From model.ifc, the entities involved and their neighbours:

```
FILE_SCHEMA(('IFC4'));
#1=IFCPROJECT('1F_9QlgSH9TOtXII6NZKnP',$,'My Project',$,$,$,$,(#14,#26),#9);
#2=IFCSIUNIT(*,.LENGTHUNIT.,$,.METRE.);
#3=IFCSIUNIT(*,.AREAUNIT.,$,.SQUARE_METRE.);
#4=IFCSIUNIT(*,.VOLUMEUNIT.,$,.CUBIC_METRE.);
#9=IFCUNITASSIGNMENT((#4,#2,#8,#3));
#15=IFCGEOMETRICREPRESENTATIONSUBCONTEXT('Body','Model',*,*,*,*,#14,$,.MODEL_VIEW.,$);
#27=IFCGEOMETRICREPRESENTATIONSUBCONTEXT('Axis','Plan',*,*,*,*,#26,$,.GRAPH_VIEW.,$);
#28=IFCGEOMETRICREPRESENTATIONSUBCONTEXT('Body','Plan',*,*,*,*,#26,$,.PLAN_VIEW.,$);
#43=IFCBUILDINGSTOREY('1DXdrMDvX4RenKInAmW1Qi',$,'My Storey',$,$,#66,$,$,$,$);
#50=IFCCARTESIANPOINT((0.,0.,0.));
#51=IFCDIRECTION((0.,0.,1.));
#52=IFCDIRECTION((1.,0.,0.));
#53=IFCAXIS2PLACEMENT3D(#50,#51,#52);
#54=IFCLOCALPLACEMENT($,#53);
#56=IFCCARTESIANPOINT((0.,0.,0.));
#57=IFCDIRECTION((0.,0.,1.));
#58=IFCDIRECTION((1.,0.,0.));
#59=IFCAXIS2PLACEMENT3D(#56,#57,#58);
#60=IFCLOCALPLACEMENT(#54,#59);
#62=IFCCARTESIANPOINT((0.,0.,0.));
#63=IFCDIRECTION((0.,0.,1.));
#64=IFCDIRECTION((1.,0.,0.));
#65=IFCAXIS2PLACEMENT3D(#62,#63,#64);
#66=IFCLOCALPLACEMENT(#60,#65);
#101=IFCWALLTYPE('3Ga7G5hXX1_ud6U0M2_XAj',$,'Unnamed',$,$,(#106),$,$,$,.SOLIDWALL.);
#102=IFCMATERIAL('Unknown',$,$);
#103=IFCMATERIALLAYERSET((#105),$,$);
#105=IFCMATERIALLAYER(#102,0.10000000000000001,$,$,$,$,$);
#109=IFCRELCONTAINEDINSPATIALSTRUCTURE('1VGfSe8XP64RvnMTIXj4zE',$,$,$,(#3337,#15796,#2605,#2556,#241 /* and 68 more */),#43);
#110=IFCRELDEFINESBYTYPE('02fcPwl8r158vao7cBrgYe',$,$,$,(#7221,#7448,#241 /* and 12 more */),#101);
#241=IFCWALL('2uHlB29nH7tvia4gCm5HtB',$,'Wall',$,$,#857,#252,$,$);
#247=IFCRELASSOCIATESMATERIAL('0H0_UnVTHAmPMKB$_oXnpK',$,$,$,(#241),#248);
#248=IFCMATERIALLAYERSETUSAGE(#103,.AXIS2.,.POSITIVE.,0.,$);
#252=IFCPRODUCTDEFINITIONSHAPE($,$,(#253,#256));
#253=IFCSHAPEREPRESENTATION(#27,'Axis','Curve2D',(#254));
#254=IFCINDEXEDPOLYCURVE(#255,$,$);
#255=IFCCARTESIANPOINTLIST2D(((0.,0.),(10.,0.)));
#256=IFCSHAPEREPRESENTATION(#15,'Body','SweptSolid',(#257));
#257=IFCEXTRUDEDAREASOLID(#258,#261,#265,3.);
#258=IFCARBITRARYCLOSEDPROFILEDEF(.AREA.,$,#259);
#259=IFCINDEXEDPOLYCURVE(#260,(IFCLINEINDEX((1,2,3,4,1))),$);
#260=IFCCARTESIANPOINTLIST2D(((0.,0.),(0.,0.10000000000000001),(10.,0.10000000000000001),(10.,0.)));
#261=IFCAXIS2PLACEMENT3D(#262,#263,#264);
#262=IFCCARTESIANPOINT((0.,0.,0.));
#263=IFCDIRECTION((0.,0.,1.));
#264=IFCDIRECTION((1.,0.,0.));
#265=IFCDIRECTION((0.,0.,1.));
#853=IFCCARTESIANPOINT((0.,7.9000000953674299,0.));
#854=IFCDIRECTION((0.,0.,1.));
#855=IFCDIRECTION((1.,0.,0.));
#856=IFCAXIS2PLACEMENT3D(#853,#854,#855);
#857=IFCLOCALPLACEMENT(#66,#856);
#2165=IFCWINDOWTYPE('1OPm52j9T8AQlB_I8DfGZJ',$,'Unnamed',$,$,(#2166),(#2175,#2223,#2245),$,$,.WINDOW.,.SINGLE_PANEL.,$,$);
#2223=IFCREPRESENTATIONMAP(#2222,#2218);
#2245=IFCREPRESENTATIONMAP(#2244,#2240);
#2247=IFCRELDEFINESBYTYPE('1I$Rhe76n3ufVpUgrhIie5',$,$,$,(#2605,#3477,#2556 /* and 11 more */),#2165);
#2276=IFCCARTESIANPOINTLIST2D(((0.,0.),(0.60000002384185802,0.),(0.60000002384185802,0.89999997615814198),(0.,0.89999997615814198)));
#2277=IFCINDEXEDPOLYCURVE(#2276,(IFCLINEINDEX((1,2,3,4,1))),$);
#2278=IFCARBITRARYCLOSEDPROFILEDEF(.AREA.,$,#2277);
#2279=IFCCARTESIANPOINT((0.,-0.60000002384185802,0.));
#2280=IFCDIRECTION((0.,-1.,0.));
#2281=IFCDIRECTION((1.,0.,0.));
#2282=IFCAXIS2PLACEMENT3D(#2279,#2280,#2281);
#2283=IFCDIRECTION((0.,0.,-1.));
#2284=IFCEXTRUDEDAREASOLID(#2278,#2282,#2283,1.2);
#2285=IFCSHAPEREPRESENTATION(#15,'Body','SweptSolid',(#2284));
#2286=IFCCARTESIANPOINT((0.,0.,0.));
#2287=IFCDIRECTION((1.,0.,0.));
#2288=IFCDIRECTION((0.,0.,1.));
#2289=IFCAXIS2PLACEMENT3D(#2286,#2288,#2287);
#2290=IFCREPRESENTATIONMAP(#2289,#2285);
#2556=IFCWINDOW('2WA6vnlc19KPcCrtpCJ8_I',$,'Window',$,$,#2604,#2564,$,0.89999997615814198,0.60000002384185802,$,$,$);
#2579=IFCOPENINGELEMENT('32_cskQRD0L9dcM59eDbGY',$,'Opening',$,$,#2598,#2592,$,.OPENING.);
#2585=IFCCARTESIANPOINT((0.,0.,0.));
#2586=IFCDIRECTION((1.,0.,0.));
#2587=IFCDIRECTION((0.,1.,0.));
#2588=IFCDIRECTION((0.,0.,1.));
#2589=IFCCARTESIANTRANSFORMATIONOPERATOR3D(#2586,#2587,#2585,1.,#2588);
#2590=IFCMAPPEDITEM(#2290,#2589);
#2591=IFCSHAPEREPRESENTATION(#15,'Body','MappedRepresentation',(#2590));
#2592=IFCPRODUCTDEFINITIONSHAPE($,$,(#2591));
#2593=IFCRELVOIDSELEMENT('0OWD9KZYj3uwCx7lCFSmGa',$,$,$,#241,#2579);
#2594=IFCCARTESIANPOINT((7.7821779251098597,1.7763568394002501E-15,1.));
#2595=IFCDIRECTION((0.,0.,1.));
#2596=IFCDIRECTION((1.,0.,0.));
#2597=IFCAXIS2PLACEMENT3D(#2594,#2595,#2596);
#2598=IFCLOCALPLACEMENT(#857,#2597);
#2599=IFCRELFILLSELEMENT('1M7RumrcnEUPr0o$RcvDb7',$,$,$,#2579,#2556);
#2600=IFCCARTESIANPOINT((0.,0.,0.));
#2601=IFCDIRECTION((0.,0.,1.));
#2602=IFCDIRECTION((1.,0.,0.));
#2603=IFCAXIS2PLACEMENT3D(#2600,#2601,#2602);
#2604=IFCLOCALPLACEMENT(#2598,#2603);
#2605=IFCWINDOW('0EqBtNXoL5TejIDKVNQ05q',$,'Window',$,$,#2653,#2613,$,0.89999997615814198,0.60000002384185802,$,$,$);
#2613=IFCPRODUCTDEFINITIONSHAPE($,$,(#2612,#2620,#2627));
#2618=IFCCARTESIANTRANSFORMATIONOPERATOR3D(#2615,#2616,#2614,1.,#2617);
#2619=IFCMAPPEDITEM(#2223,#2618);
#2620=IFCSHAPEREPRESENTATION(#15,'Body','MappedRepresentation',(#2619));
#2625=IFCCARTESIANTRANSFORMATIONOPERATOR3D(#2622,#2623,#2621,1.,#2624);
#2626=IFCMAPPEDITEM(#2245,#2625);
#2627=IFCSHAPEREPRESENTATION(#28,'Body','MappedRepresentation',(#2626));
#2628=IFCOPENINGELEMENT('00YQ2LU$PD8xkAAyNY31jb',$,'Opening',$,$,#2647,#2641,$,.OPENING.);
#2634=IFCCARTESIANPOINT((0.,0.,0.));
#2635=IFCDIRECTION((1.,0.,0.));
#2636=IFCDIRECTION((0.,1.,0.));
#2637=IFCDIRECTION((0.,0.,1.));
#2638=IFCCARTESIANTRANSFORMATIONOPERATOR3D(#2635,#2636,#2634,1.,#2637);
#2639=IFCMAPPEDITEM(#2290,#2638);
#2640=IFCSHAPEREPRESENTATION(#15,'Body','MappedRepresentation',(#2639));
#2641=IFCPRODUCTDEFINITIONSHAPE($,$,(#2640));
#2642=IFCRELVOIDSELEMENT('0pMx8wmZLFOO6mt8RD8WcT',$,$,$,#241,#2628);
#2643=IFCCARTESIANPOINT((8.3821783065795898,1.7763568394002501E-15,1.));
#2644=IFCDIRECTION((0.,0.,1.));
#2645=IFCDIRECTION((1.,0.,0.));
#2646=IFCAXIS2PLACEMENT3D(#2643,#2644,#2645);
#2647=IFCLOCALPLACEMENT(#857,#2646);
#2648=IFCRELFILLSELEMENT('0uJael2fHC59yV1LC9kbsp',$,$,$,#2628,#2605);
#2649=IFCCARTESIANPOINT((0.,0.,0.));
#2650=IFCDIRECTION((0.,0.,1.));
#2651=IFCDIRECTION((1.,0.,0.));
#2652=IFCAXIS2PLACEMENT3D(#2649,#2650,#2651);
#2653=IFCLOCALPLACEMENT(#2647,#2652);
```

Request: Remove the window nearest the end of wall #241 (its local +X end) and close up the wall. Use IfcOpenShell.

```python
import ifcopenshell
import ifcopenshell.api.feature
import ifcopenshell.api.root
import ifcopenshell.geom
import ifcopenshell.util.shape

model = ifcopenshell.open("model.ifc")
settings = ifcopenshell.geom.settings()


def volume(element):
    """Net volume in cubic metres, openings subtracted."""
    shape = ifcopenshell.geom.create_shape(settings, element)
    return ifcopenshell.util.shape.get_volume(shape.geometry)


window = model.by_guid("0EqBtNXoL5TejIDKVNQ05q")
opening = window.FillsVoids[0].RelatingOpeningElement
wall = opening.VoidsElements[0].RelatingBuildingElement
before = volume(wall)

ifcopenshell.api.root.remove_product(model, product=window)
ifcopenshell.api.feature.remove_feature(model, feature=opening)

after = volume(wall)

print(f"wall volume {before:.3f} -> {after:.3f} m3")

model.write("model_edited.ifc")
```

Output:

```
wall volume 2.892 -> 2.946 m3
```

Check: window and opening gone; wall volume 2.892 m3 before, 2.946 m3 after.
